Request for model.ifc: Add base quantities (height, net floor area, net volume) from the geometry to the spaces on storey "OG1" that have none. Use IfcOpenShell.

First a look at what the model holds.

```python
import ifcopenshell
import ifcopenshell.util.element
import ifcopenshell.util.unit

model = ifcopenshell.open("model.ifc")
print(model.schema)
for unit_type in ("LENGTHUNIT", "AREAUNIT", "VOLUMEUNIT"):
    print(unit_type, ifcopenshell.util.unit.calculate_unit_scale(model, unit_type))
storey = next(s for s in model.by_type("IfcBuildingStorey") if s.Name == "OG1")
spaces = [e for e in ifcopenshell.util.element.get_decomposition(storey) if e.is_a("IfcSpace")]
for e in sorted(spaces, key=lambda e: e.id()):
    print(e.id(), e.is_a(), e.Name, list(ifcopenshell.util.element.get_psets(e, qtos_only=True)), sep=" | ")
```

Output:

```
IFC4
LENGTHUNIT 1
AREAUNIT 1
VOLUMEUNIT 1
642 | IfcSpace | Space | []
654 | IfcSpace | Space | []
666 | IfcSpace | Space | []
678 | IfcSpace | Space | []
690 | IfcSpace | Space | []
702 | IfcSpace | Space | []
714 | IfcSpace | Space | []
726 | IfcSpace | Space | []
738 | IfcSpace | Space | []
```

```python
import ifcopenshell
import ifcopenshell.api.pset
import ifcopenshell.geom
import ifcopenshell.util.element
import ifcopenshell.util.shape
import ifcopenshell.util.unit

model = ifcopenshell.open("model.ifc")
unit_scale = ifcopenshell.util.unit.calculate_unit_scale(model)
area_scale = ifcopenshell.util.unit.calculate_unit_scale(model, "AREAUNIT")
volume_scale = ifcopenshell.util.unit.calculate_unit_scale(model, "VOLUMEUNIT")
settings = ifcopenshell.geom.settings()

storey = next(s for s in model.by_type("IfcBuildingStorey") if s.Name == "OG1")
spaces = [e for e in ifcopenshell.util.element.get_decomposition(storey) if e.is_a("IfcSpace")]

for e in sorted(spaces, key=lambda e: e.id()):
    if ifcopenshell.util.element.get_psets(e, qtos_only=True, should_inherit=False):
        continue
    # Geometry comes back in metres, in the element's own axes.
    shape = ifcopenshell.geom.create_shape(settings, e)
    values = {
        "Height": ifcopenshell.util.shape.get_z(shape.geometry) / unit_scale,
        "NetFloorArea": ifcopenshell.util.shape.get_footprint_area(shape.geometry) / area_scale,
        "NetVolume": ifcopenshell.util.shape.get_volume(shape.geometry) / volume_scale,
    }
    qto = ifcopenshell.api.pset.add_qto(model, product=e, name="Qto_SpaceBaseQuantities")
    ifcopenshell.api.pset.edit_qto(model, qto=qto, properties=values)
    print(e.id(), {k: round(v, 3) for k, v in values.items()})

model.write("model_rev.ifc")
```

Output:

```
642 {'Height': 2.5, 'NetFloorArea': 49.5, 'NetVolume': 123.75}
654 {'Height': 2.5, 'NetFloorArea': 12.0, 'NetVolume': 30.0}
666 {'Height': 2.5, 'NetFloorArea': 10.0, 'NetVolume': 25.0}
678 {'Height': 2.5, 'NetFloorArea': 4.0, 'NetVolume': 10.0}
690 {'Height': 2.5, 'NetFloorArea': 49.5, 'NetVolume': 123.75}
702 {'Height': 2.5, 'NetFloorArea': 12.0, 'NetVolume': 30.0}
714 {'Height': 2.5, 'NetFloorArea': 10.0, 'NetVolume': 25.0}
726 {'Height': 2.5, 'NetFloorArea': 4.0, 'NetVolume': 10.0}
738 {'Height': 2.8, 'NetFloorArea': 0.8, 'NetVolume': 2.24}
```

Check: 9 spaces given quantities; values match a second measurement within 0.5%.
